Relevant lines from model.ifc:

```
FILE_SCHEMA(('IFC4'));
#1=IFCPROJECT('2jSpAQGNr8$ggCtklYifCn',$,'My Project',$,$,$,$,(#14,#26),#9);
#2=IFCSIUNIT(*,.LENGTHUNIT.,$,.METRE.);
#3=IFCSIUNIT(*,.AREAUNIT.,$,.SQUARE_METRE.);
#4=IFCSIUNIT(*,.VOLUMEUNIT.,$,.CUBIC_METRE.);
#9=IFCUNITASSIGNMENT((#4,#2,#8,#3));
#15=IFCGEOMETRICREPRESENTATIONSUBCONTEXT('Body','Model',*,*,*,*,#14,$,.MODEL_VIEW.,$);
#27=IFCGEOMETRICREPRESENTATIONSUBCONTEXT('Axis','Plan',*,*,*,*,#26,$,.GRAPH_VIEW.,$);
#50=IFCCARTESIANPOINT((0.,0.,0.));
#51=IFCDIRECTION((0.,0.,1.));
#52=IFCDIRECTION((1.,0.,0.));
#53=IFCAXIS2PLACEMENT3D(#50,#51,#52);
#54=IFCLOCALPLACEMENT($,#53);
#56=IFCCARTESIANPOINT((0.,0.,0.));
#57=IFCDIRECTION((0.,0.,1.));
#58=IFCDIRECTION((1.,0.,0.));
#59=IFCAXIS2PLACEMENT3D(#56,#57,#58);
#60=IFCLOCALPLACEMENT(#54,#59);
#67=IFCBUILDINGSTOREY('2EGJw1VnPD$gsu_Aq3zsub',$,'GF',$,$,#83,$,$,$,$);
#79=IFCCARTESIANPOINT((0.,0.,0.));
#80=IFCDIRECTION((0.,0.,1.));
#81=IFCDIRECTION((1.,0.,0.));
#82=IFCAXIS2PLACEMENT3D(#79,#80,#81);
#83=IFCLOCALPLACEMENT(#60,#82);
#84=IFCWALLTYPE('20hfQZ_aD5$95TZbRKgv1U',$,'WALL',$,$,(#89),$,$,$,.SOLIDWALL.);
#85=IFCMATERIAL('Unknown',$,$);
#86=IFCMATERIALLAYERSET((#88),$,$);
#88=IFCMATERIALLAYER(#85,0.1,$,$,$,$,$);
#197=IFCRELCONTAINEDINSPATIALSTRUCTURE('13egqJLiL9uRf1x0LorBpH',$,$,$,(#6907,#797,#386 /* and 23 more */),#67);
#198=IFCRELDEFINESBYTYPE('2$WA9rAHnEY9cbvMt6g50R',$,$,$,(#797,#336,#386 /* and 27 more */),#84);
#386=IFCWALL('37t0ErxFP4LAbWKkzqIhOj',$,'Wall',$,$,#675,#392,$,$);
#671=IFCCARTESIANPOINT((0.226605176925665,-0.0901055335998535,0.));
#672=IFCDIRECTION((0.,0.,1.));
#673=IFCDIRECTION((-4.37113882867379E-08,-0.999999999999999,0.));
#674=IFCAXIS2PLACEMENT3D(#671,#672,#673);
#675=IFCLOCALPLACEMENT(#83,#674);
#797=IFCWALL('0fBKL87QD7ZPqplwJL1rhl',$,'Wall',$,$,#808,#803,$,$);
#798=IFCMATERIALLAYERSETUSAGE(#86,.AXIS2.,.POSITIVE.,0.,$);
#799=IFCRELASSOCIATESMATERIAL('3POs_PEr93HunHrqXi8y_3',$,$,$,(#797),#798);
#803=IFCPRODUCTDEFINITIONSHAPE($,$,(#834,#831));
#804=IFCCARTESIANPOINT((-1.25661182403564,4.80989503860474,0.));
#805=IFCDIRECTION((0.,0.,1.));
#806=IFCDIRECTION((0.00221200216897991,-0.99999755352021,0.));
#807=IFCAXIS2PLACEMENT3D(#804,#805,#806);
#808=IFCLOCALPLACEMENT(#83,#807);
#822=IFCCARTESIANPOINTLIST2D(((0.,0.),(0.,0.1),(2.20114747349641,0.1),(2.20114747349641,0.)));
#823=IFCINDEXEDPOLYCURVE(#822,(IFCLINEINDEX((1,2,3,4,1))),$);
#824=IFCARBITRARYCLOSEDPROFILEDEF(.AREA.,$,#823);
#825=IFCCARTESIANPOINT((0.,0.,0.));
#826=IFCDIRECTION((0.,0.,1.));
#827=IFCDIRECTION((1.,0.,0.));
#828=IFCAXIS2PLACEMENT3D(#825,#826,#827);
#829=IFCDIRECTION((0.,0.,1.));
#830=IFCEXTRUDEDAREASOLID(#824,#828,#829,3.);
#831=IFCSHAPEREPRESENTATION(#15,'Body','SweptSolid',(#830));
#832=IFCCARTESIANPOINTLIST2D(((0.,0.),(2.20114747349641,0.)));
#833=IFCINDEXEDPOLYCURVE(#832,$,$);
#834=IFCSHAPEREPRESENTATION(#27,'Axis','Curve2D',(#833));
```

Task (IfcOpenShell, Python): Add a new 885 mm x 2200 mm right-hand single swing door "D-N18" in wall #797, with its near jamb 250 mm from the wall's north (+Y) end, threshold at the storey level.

```python
import numpy as np
import ifcopenshell
import ifcopenshell.api.feature
import ifcopenshell.api.geometry
import ifcopenshell.api.root
import ifcopenshell.api.spatial
import ifcopenshell.geom
import ifcopenshell.util.element
import ifcopenshell.util.placement
import ifcopenshell.util.representation
import ifcopenshell.util.shape
import ifcopenshell.util.unit

model = ifcopenshell.open("model.ifc")
unit_scale = ifcopenshell.util.unit.calculate_unit_scale(model)
settings = ifcopenshell.geom.settings()


def volume(element):
    """Net volume in cubic metres, openings subtracted."""
    shape = ifcopenshell.geom.create_shape(settings, element)
    return ifcopenshell.util.shape.get_volume(shape.geometry)


wall = model.by_id(797)
storey = ifcopenshell.util.element.get_container(wall, ifc_class="IfcBuildingStorey")
context = ifcopenshell.util.representation.get_context(model, "Model", "Body", "MODEL_VIEW")
before = volume(wall)

width, height, from_end, sill = 0.885, 2.2, 0.25, 0.0  # metres

# The wall runs along its own X axis, and the end named is its -X end.
wall_shape = ifcopenshell.geom.create_shape(settings, wall)
x, y, z = ifcopenshell.util.shape.get_vertices(wall_shape.geometry).T
start = x.min() + from_end
face, thickness = float(y.min()), float(y.max() - y.min())
wall_matrix = ifcopenshell.util.placement.get_local_placement(wall.ObjectPlacement)
level = ifcopenshell.util.placement.get_local_placement(storey.ObjectPlacement)[2, 3]


def in_wall(x, y):
    """Placement at x, y metres in the wall's axes, at sill height."""
    matrix = wall_matrix.copy()
    matrix[:, 3] = wall_matrix @ np.array([x / unit_scale, y / unit_scale, 0.0, 1.0])
    matrix[2, 3] = level + sill / unit_scale
    return matrix


# Opening: a box that overshoots both wall faces by 50 mm.
opening = ifcopenshell.api.root.create_entity(model, ifc_class="IfcOpeningElement", predefined_type="OPENING")
box = ifcopenshell.api.geometry.add_wall_representation(
    model, context=context, length=width, height=height, thickness=thickness + 0.1
)
ifcopenshell.api.geometry.assign_representation(model, product=opening, representation=box)
ifcopenshell.api.geometry.edit_object_placement(model, product=opening, matrix=in_wall(start, face - 0.05), is_si=False)
ifcopenshell.api.feature.add_feature(model, feature=opening, element=wall)

door = ifcopenshell.api.root.create_entity(model, ifc_class="IfcDoor", name="D-N18", predefined_type="DOOR")
door.OverallWidth, door.OverallHeight = width / unit_scale, height / unit_scale
door.OperationType = "SINGLE_SWING_RIGHT"
body = ifcopenshell.api.geometry.add_door_representation(
    model,
    context=context,
    overall_width=door.OverallWidth,
    overall_height=door.OverallHeight,
    operation_type="SINGLE_SWING_RIGHT",
    lining_properties={"LiningDepth": thickness / unit_scale, "ThresholdDepth": thickness / unit_scale},
)
ifcopenshell.api.geometry.assign_representation(model, product=door, representation=body)
ifcopenshell.api.spatial.assign_container(model, products=[door], relating_structure=storey)
ifcopenshell.api.feature.add_filling(model, opening=opening, element=door)

# The lining spans the wall, so the door starts at the wall face.
ifcopenshell.api.geometry.edit_object_placement(model, product=door, matrix=in_wall(start, face), is_si=False)

after = volume(wall)

print(f"wall volume {before:.3f} -> {after:.3f} m3")

model.write("model_edited.ifc")
```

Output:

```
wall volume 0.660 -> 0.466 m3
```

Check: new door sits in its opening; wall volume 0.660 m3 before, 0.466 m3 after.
